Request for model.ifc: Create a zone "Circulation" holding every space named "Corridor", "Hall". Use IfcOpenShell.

First a look at what the model holds.

```python
import ifcopenshell

model = ifcopenshell.open("model.ifc")
print(model.schema)
seen = {}
for space in model.by_type("IfcSpace"):
    seen[space.LongName] = seen.get(space.LongName, 0) + 1
for name, count in sorted(seen.items(), key=str):
    print(count, "x", name)
print("zones:", [z.Name for z in model.by_type("IfcZone")][:20])
```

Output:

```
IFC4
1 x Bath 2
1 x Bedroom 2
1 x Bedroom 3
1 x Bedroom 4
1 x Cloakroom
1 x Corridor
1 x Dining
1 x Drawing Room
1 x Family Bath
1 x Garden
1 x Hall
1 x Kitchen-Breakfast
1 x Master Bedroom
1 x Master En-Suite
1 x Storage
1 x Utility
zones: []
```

```python
import ifcopenshell
import ifcopenshell.api.group
import ifcopenshell.api.root

model = ifcopenshell.open("model.ifc")

names = {"Corridor", "Hall"}
spaces = [s for s in model.by_type("IfcSpace") if s.LongName in names]

zone = ifcopenshell.api.root.create_entity(model, ifc_class="IfcZone", name="Circulation")
ifcopenshell.api.group.assign_group(model, products=spaces, group=zone)
print(len(spaces), "spaces in", zone.Name)

model.write("model_edited.ifc")
```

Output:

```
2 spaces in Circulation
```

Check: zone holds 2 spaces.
